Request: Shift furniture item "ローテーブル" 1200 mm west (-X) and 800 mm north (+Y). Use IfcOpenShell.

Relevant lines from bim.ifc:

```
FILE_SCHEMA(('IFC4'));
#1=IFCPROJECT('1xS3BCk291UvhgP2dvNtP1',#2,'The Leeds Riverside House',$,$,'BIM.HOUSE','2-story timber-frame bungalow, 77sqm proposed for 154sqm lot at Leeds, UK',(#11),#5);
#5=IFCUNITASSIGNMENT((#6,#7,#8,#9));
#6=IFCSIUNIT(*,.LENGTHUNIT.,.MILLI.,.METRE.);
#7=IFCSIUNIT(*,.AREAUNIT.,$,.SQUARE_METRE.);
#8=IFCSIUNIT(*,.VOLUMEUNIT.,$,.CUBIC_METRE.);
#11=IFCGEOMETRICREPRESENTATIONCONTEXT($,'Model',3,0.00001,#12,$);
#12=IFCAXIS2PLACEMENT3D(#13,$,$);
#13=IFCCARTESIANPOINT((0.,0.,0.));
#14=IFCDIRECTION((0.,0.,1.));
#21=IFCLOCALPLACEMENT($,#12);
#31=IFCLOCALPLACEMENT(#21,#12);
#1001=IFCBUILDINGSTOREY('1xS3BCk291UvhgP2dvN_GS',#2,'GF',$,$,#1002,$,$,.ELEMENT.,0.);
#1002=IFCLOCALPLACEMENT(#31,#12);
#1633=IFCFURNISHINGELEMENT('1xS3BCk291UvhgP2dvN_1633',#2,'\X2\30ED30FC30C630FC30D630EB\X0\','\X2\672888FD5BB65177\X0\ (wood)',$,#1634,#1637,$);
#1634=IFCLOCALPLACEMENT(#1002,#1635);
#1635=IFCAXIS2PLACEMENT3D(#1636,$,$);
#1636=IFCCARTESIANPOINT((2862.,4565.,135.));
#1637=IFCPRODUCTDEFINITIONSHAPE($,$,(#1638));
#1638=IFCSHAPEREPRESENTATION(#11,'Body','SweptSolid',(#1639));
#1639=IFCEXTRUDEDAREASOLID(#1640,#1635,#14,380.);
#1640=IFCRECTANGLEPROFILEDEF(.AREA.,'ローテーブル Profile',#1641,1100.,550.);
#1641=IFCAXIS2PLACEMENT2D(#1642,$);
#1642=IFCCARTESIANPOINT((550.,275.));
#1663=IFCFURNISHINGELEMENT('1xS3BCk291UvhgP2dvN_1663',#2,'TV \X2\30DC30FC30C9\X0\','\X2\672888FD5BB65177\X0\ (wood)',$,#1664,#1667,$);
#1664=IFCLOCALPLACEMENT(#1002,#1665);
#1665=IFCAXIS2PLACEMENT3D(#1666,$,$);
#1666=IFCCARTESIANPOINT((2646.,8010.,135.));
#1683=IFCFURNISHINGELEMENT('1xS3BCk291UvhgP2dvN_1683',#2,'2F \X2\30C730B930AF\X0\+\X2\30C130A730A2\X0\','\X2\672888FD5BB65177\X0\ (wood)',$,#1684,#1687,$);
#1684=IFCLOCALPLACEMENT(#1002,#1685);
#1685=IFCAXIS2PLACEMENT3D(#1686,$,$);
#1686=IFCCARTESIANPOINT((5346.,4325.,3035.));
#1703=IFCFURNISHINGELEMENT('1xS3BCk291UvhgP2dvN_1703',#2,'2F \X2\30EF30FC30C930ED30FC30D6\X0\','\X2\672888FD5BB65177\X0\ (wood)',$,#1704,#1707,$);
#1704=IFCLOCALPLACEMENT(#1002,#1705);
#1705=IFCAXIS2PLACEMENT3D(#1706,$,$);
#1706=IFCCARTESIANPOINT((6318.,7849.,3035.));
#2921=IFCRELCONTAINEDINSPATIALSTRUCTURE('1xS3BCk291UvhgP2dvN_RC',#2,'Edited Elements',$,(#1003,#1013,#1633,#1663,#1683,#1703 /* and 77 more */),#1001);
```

```python
import ifcopenshell
import ifcopenshell.api.geometry
import ifcopenshell.util.placement
import ifcopenshell.util.unit

model = ifcopenshell.open("bim.ifc")
unit_scale = ifcopenshell.util.unit.calculate_unit_scale(model)

item = model.by_guid("1xS3BCk291UvhgP2dvN_1633")
matrix = ifcopenshell.util.placement.get_local_placement(item.ObjectPlacement)
matrix[0, 3] -= 1.2 / unit_scale
matrix[1, 3] += 0.8 / unit_scale
ifcopenshell.api.geometry.edit_object_placement(model, product=item, matrix=matrix, is_si=False)

print(ifcopenshell.util.placement.get_local_placement(item.ObjectPlacement).round(3) + 0.0)

model.write("bim_updated.ifc")
```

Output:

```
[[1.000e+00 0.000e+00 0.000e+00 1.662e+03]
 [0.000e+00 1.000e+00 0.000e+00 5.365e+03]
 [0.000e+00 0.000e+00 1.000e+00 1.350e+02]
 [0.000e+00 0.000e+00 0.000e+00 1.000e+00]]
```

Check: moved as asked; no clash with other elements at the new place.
